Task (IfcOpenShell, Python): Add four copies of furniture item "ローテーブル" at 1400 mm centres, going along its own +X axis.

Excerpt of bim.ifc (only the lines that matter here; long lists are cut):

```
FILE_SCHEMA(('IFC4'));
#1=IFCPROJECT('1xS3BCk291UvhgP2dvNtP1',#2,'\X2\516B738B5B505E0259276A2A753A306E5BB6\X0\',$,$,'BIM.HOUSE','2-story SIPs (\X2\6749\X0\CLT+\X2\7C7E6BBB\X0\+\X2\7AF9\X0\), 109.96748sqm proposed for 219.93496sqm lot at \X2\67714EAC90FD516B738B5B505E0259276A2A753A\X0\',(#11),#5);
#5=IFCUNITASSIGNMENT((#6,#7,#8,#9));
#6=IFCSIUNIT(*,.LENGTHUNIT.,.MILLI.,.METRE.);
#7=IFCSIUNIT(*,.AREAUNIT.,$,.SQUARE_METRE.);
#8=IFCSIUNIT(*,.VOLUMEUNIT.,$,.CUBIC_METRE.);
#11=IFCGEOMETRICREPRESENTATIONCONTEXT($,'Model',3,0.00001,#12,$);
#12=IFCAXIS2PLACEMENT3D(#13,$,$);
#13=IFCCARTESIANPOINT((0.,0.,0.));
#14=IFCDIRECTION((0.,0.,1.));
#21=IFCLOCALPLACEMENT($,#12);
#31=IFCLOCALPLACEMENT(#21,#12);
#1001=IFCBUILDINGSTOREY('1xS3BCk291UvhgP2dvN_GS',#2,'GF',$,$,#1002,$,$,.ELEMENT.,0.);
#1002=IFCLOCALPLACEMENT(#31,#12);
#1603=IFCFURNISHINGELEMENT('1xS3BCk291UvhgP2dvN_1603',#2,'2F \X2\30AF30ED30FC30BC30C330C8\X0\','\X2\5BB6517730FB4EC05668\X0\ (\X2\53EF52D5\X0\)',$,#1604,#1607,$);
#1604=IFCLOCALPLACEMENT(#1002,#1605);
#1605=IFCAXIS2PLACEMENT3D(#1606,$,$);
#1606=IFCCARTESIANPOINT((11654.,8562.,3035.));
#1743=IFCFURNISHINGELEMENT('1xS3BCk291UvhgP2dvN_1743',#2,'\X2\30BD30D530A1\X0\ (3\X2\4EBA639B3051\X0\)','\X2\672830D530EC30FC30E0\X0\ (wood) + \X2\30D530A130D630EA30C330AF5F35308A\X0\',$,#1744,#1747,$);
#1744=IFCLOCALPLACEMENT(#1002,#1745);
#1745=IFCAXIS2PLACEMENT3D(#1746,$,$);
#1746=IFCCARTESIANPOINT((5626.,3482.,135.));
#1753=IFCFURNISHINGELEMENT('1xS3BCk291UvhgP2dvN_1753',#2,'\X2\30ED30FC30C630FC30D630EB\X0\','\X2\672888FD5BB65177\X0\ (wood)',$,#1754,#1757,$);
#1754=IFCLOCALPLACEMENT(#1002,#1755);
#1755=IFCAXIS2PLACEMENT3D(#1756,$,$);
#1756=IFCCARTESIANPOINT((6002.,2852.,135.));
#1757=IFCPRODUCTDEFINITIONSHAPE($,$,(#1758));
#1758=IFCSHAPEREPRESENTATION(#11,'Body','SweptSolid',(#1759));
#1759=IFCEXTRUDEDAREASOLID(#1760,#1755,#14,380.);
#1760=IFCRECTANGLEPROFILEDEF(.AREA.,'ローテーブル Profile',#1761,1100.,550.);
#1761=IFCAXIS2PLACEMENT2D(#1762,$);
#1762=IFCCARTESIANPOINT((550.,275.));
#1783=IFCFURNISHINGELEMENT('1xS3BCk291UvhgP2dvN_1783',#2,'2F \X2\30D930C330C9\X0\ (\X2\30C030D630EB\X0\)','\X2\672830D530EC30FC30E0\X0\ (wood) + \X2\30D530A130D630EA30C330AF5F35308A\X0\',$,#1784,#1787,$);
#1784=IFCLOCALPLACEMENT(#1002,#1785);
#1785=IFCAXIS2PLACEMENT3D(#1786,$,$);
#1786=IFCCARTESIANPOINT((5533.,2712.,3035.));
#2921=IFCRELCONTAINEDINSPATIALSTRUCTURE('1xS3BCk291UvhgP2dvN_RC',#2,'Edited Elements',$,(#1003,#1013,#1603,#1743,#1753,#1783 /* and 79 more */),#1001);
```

```python
import ifcopenshell
import ifcopenshell.api.geometry
import ifcopenshell.api.root
import ifcopenshell.util.element
import ifcopenshell.util.placement

model = ifcopenshell.open("bim.ifc")


def reuse_history(source, copy):
    """copy_class also copies each property set's owner history, people and application; keep the originals."""
    for rel in copy.IsDefinedBy:
        if rel.is_a("IfcRelDefinesByProperties") and (history := rel.RelatingPropertyDefinition.OwnerHistory):
            rel.RelatingPropertyDefinition.OwnerHistory = source.OwnerHistory
            ifcopenshell.util.element.remove_deep2(model, history)


source = model.by_guid("1xS3BCk291UvhgP2dvN_1753")
base = ifcopenshell.util.placement.get_local_placement(source.ObjectPlacement)
step = base[:3, 0] * 1400.0

for i in range(1, 5):
    copy = ifcopenshell.api.root.copy_class(model, product=source)
    copy.Representation = ifcopenshell.util.element.copy_deep(
        model, source.Representation, exclude=["IfcGeometricRepresentationContext", "IfcRepresentationMap"]
    )
    reuse_history(source, copy)
    matrix = base.copy()
    matrix[:3, 3] += i * step
    print("added at", matrix[:3, 3].round(3) + 0.0)
    ifcopenshell.api.geometry.edit_object_placement(model, product=copy, matrix=matrix, is_si=False)

model.write("bim-out.ifc")
```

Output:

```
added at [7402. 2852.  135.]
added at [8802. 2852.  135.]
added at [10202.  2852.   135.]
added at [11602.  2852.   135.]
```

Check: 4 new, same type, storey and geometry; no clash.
